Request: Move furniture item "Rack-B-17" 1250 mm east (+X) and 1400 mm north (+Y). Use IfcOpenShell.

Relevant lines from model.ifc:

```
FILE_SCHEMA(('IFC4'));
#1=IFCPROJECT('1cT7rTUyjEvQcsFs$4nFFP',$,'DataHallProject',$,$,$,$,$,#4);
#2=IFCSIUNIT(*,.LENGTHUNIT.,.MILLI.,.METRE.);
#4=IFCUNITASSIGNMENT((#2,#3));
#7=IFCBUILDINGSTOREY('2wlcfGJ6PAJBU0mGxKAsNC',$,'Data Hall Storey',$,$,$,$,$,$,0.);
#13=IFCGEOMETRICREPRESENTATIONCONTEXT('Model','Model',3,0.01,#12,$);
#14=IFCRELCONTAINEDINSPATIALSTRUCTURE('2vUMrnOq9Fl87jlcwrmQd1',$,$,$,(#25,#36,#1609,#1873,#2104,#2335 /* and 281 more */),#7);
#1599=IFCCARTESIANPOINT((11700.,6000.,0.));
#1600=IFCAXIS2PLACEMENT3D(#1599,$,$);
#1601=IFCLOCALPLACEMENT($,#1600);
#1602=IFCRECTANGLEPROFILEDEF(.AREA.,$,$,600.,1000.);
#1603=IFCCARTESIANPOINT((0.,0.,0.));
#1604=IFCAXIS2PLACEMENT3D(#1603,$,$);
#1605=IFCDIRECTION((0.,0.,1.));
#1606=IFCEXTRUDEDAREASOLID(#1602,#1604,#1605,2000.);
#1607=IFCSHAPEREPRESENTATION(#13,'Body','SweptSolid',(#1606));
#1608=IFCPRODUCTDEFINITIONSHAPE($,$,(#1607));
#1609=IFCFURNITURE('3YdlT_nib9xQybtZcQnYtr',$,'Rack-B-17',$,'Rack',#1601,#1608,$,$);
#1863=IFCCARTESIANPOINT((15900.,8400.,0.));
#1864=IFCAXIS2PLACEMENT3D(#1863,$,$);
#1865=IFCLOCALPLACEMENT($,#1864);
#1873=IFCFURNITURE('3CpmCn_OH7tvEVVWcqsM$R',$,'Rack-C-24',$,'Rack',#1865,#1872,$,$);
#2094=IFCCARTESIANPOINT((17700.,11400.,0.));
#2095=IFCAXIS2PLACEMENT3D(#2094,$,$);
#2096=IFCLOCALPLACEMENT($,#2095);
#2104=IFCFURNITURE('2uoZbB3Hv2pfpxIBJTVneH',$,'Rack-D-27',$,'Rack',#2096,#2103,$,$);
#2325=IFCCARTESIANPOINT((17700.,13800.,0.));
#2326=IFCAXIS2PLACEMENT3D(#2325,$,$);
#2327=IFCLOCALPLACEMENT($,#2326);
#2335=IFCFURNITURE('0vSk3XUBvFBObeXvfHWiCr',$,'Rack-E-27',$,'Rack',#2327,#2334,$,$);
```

```python
import ifcopenshell
import ifcopenshell.api.geometry
import ifcopenshell.util.placement

model = ifcopenshell.open("model.ifc")

item = model.by_guid("3YdlT_nib9xQybtZcQnYtr")
matrix = ifcopenshell.util.placement.get_local_placement(item.ObjectPlacement)
matrix[0, 3] += 1250.0
matrix[1, 3] += 1400.0
ifcopenshell.api.geometry.edit_object_placement(model, product=item, matrix=matrix, is_si=False)

print(ifcopenshell.util.placement.get_local_placement(item.ObjectPlacement).round(3) + 0.0)

model.write("model-out.ifc")
```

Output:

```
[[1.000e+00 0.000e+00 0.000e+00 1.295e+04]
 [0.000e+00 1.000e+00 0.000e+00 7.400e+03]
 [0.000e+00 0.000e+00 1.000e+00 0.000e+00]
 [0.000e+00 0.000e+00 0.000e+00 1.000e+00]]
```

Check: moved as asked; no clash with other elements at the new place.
